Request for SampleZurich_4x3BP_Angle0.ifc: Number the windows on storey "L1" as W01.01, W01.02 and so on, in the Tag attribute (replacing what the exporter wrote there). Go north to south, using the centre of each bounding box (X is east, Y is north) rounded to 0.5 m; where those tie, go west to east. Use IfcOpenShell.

First a look at what the model holds.

```python
import ifcopenshell
import ifcopenshell.util.element
import ifcopenshell.util.placement

model = ifcopenshell.open("SampleZurich_4x3BP_Angle0.ifc")
print(model.schema)
storey = next(s for s in model.by_type("IfcBuildingStorey") if s.Name == "L1")
windows = [e for e in ifcopenshell.util.element.get_decomposition(storey) if e.is_a("IfcWindow")]
for e in sorted(windows, key=lambda e: e.id()):
    origin = ifcopenshell.util.placement.get_local_placement(e.ObjectPlacement)[:3, 3]
    print(e.id(), e.Tag, e.Name, origin.round(2) + 0.0, sep=" | ")
```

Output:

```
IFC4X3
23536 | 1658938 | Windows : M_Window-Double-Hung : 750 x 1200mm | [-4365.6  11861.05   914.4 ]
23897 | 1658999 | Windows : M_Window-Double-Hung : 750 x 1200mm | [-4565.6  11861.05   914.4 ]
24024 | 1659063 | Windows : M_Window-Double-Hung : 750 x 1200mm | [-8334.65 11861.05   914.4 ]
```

```python
import ifcopenshell
import ifcopenshell.geom
import ifcopenshell.util.element
import ifcopenshell.util.shape

model = ifcopenshell.open("SampleZurich_4x3BP_Angle0.ifc")
settings = ifcopenshell.geom.settings()
settings.set("use-world-coords", True)


def centre(element):
    shape = ifcopenshell.geom.create_shape(settings, element)
    return ifcopenshell.util.shape.get_bbox_centroid(shape.geometry)


storey = next(s for s in model.by_type("IfcBuildingStorey") if s.Name == "L1")
windows = [e for e in ifcopenshell.util.element.get_decomposition(storey) if e.is_a("IfcWindow")]

# Insertion points can sit at a corner or the storey origin, so sort by the geometry (in metres).
centres = {e: centre(e) for e in windows}
windows.sort(key=lambda e: (-round(centres[e][1] / 0.5), centres[e][0]))

for i, e in enumerate(windows, start=1):
    number = f"W01.{i:02d}"
    e.Tag = number
    print(e.id(), number)

model.write("SampleZurich_4x3BP_Angle0-out.ifc")
```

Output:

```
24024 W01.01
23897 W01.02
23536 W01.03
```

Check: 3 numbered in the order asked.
